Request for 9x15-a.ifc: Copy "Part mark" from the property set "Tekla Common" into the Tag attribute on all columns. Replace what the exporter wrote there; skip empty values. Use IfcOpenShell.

First a look at what the model holds.

```python
import ifcopenshell
import ifcopenshell.util.element

model = ifcopenshell.open("9x15-a.ifc")
print(model.schema)
columns = model.by_type("IfcColumn")
print(len(columns), "columns")
for e in columns[:8]:
    source = ifcopenshell.util.element.get_pset(e, "Tekla Common", "Part mark")
    target = e.Tag
    print(e.id(), repr(source), repr(target), sep=" | ")
```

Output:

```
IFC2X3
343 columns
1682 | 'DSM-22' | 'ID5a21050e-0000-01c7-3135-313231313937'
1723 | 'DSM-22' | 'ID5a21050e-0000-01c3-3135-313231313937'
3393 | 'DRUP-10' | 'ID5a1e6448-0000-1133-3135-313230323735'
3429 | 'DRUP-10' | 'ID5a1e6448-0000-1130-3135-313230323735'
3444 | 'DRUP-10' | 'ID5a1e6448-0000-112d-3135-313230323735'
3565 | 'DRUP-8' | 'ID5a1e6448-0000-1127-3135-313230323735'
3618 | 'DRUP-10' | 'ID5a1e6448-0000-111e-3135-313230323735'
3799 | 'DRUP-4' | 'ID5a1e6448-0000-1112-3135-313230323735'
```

```python
import ifcopenshell
import ifcopenshell.util.element

model = ifcopenshell.open("9x15-a.ifc")

count = 0
for e in model.by_type("IfcColumn"):
    value = ifcopenshell.util.element.get_pset(e, "Tekla Common", "Part mark")
    current = e.Tag
    if not value or not value.strip() or current == value:
        continue
    e.Tag = value
    count += 1

print(count, "columns updated")

model.write("9x15-a_updated.ifc")
```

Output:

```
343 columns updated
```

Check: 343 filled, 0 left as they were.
